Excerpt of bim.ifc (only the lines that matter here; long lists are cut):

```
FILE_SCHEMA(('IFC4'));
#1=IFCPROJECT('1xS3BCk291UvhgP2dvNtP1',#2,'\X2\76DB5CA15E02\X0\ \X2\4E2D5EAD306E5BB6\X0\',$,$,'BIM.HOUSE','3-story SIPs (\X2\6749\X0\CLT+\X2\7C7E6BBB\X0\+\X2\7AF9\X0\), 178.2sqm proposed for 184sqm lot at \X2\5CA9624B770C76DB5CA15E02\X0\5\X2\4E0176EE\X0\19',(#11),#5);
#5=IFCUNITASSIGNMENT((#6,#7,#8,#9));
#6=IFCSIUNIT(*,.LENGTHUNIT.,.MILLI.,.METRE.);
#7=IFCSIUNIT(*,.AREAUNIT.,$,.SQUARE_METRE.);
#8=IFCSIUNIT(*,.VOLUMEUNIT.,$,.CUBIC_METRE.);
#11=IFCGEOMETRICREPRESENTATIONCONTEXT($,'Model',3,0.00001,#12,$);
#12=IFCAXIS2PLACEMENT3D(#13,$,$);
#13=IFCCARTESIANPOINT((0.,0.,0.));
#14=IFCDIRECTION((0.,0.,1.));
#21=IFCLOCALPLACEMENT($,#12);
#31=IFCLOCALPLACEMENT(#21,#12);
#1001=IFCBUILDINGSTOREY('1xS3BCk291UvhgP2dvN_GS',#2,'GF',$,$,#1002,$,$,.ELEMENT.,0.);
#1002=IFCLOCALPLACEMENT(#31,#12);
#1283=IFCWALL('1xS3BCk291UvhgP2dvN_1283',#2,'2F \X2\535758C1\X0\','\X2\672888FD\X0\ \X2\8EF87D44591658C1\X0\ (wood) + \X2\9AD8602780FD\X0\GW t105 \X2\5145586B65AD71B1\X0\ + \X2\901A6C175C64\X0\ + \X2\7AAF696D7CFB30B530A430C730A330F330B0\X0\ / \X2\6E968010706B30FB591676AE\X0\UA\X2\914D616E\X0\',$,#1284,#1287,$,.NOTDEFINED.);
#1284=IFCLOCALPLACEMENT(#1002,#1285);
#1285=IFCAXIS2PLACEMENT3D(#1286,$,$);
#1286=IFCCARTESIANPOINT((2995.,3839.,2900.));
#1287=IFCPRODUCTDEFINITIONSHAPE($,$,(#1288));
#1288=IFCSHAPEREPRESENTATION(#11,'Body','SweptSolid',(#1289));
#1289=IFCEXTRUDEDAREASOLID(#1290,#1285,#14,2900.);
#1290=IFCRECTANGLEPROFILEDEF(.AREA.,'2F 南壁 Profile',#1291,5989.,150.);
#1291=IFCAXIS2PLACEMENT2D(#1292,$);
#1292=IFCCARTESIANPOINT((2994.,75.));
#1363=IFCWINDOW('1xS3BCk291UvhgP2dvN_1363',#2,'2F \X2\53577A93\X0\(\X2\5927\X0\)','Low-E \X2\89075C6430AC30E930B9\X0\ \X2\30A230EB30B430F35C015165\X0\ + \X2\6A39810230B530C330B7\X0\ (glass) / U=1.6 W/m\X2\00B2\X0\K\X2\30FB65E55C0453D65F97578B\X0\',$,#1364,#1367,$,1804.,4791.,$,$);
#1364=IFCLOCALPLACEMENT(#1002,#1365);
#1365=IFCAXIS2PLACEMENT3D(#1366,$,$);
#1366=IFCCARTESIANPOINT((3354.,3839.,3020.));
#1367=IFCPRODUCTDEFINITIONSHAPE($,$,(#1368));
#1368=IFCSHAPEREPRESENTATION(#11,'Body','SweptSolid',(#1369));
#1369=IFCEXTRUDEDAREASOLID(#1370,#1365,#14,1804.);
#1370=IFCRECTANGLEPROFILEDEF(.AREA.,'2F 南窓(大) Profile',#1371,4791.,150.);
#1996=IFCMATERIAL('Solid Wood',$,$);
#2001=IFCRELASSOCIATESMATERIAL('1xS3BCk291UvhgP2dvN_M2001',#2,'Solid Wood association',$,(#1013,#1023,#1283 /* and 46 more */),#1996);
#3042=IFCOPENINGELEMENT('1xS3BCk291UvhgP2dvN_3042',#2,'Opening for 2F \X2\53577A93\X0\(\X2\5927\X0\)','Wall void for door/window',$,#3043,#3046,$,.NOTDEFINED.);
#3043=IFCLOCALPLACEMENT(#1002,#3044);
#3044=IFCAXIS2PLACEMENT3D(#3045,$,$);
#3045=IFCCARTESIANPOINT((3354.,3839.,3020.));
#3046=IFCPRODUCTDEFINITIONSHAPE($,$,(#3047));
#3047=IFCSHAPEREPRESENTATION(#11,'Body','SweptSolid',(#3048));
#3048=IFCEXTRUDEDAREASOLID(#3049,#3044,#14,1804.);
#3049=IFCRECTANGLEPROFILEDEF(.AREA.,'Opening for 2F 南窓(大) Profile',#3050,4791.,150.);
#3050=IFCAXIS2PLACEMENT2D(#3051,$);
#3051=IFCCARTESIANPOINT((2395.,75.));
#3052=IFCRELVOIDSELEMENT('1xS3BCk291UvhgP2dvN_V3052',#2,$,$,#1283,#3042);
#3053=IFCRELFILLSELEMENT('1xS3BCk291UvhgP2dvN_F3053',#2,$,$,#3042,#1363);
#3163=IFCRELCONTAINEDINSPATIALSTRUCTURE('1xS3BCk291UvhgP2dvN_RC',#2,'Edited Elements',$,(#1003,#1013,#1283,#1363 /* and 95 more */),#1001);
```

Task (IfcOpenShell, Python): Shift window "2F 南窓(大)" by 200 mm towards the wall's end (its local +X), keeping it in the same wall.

```python
import ifcopenshell
import ifcopenshell.api.geometry
import ifcopenshell.util.placement
import ifcopenshell.util.unit

model = ifcopenshell.open("bim.ifc")
unit_scale = ifcopenshell.util.unit.calculate_unit_scale(model)

window = model.by_guid("1xS3BCk291UvhgP2dvN_1363")
opening = window.FillsVoids[0].RelatingOpeningElement
wall = opening.VoidsElements[0].RelatingBuildingElement

wall_matrix = ifcopenshell.util.placement.get_local_placement(wall.ObjectPlacement)
shift = wall_matrix[:3, 0] * 0.2 / unit_scale
before = ifcopenshell.util.placement.get_local_placement(window.ObjectPlacement)[:3, 3].copy()

# The window is not placed relative to its opening, so move both.
for product in (opening, window):
    matrix = ifcopenshell.util.placement.get_local_placement(product.ObjectPlacement)
    matrix[:3, 3] += shift
    ifcopenshell.api.geometry.edit_object_placement(model, product=product, matrix=matrix, is_si=False)

after = ifcopenshell.util.placement.get_local_placement(window.ObjectPlacement)[:3, 3]
print("window moved by", (after - before).round(3) + 0.0)

model.write("bim-out.ifc")
```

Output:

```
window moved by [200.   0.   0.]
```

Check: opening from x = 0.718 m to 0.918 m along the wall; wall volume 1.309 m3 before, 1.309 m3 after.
